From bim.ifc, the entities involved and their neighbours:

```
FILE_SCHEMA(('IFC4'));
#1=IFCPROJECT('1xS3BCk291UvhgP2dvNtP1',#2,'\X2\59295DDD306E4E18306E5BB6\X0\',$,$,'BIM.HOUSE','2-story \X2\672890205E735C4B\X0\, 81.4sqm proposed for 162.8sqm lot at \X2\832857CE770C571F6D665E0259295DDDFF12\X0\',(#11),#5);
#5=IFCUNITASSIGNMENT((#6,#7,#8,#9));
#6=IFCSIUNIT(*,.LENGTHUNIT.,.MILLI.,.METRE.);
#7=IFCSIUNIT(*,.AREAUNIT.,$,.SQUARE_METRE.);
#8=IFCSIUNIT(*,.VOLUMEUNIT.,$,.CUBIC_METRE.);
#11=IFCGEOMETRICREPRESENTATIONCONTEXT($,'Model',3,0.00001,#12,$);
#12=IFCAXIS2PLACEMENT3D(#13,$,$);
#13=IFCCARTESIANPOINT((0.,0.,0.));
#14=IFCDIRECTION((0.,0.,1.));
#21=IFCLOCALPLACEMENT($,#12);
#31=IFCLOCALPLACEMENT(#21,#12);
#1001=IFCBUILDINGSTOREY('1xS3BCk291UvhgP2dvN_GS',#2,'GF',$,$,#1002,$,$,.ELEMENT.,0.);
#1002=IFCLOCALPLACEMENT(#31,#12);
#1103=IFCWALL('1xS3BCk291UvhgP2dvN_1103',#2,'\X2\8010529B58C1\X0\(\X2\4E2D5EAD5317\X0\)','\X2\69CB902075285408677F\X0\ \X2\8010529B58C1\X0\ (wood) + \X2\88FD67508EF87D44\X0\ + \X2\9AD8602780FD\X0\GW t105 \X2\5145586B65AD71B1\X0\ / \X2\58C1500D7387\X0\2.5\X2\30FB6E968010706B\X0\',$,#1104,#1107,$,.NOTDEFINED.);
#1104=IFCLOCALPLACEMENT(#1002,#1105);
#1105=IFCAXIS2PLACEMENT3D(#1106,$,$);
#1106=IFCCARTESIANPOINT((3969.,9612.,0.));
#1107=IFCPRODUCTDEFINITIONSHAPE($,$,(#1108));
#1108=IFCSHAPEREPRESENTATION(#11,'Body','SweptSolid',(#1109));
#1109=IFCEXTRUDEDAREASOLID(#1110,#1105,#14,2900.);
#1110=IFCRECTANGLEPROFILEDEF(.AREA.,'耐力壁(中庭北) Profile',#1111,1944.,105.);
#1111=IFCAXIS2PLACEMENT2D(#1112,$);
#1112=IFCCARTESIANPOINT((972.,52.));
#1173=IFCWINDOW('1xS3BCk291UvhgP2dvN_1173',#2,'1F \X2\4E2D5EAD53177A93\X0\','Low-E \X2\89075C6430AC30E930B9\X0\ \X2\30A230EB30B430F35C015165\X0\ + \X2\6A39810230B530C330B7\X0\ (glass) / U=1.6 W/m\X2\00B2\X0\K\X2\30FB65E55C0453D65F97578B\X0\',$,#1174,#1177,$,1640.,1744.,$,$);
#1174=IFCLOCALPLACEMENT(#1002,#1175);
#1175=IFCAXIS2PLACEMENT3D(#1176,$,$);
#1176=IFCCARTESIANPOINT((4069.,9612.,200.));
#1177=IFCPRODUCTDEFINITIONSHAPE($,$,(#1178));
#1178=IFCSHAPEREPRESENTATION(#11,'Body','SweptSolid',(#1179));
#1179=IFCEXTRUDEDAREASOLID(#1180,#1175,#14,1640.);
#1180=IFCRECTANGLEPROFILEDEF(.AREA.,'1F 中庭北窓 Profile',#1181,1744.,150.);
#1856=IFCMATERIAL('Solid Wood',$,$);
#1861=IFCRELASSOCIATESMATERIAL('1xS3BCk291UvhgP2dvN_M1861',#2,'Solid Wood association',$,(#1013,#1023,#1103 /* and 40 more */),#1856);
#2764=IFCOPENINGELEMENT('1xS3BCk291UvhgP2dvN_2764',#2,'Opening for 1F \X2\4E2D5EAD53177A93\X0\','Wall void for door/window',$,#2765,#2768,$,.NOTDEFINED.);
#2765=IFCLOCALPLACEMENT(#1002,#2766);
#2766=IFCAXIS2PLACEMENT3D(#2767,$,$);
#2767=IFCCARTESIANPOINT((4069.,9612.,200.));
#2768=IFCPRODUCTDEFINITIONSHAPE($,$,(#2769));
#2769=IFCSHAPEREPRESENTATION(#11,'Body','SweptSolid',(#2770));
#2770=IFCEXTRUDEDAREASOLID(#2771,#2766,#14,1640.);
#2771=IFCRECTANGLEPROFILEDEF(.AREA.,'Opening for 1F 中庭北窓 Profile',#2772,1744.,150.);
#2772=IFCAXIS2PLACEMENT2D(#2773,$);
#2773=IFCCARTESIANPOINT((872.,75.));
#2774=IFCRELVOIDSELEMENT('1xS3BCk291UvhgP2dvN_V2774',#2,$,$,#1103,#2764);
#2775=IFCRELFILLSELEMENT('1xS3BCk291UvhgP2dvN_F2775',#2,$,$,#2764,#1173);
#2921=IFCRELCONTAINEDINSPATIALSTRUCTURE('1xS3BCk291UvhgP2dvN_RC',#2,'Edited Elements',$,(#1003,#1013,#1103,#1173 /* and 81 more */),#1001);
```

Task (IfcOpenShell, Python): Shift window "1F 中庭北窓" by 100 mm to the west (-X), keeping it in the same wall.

```python
import ifcopenshell
import ifcopenshell.api.geometry
import ifcopenshell.util.placement
import ifcopenshell.util.unit

model = ifcopenshell.open("bim.ifc")
unit_scale = ifcopenshell.util.unit.calculate_unit_scale(model)

window = model.by_guid("1xS3BCk291UvhgP2dvN_1173")
opening = window.FillsVoids[0].RelatingOpeningElement
wall = opening.VoidsElements[0].RelatingBuildingElement

wall_matrix = ifcopenshell.util.placement.get_local_placement(wall.ObjectPlacement)
shift = wall_matrix[:3, 0] * -0.1 / unit_scale
before = ifcopenshell.util.placement.get_local_placement(window.ObjectPlacement)[:3, 3].copy()

# The window is not placed relative to its opening, so move both.
for product in (opening, window):
    matrix = ifcopenshell.util.placement.get_local_placement(product.ObjectPlacement)
    matrix[:3, 3] += shift
    ifcopenshell.api.geometry.edit_object_placement(model, product=product, matrix=matrix, is_si=False)

after = ifcopenshell.util.placement.get_local_placement(window.ObjectPlacement)[:3, 3]
print("window moved by", (after - before).round(3) + 0.0)

model.write("bim_v2.ifc")
```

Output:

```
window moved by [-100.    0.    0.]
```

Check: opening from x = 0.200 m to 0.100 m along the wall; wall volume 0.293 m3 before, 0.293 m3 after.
